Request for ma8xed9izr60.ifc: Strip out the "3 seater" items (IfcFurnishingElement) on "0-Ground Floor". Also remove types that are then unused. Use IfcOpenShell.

First a look at what the model holds.

```python
import ifcopenshell
import ifcopenshell.util.element

model = ifcopenshell.open("ma8xed9izr60.ifc")
print(model.schema)
storey = next(s for s in model.by_type("IfcBuildingStorey") if s.Name == "0-Ground Floor")
furniture = [e for e in ifcopenshell.util.element.get_decomposition(storey) if e.is_a("IfcFurnishingElement")]
seen = {}
for e in furniture:
    element_type = ifcopenshell.util.element.get_type(e)
    name = element_type.Name if element_type not in (None, e) else None
    seen[name] = seen.get(name, 0) + 1
for name, count in sorted(seen.items(), key=str):
    print(count, "x", name)
```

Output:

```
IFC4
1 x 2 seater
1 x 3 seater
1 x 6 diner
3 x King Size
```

```python
import ifcopenshell
import ifcopenshell.api.root
import ifcopenshell.util.element

model = ifcopenshell.open("ma8xed9izr60.ifc")

storey = next(s for s in model.by_type("IfcBuildingStorey") if s.Name == "0-Ground Floor")
furniture = [e for e in ifcopenshell.util.element.get_decomposition(storey) if e.is_a("IfcFurnishingElement")]
targets = [e for e in furniture if (t := ifcopenshell.util.element.get_type(e)) not in (None, e) and t.Name == "3 seater"]
types = {ifcopenshell.util.element.get_type(e) for e in targets} - {None, *targets}

for e in targets:
    ifcopenshell.api.root.remove_product(model, product=e)
print(len(targets), "removed")

unused = [t for t in types if not ifcopenshell.util.element.get_types(t)]
for t in unused:
    ifcopenshell.api.root.remove_product(model, product=t)
print(len(unused), "unused types removed")

model.write("ma8xed9izr60_edited.ifc")
```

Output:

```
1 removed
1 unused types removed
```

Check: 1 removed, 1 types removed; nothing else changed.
